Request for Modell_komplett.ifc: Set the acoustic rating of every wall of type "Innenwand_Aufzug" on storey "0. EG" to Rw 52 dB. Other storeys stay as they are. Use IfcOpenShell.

First a look at what the model holds.

```python
import ifcopenshell
import ifcopenshell.util.element

model = ifcopenshell.open("Modell_komplett.ifc")
print(model.schema)
storey = next(s for s in model.by_type("IfcBuildingStorey") if s.Name == "0. EG")
walls = [e for e in ifcopenshell.util.element.get_decomposition(storey) if e.is_a("IfcWall")]
seen = {}
for e in walls:
    element_type = ifcopenshell.util.element.get_type(e)
    key = (element_type.Name if element_type != e and element_type else None, ifcopenshell.util.element.get_pset(e, "Pset_WallCommon", "AcousticRating"))
    seen[key] = seen.get(key, 0) + 1
for (name, value), count in sorted(seen.items(), key=str):
    print(count, "x", name, "|", value)
```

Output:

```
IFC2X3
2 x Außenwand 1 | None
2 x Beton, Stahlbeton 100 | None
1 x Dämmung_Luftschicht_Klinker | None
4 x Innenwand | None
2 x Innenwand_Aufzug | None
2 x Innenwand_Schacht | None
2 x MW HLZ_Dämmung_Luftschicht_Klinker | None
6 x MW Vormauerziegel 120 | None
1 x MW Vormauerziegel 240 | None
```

```python
import ifcopenshell
import ifcopenshell.api.pset
import ifcopenshell.util.element

model = ifcopenshell.open("Modell_komplett.ifc")

storey = next(s for s in model.by_type("IfcBuildingStorey") if s.Name == "0. EG")
walls = [e for e in ifcopenshell.util.element.get_decomposition(storey) if e.is_a("IfcWall")]

count = 0
for e in walls:
    element_type = ifcopenshell.util.element.get_type(e)
    if element_type in (None, e) or element_type.Name != "Innenwand_Aufzug":
        continue
    # add_pset returns the element's existing set when there is one.
    pset = ifcopenshell.api.pset.add_pset(model, product=e, name="Pset_WallCommon")
    ifcopenshell.api.pset.edit_pset(model, pset=pset, properties={"AcousticRating": "Rw 52 dB"})
    count += 1

print(count, "walls updated")

model.write("Modell_komplett_v2.ifc")
```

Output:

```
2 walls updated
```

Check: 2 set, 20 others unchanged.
